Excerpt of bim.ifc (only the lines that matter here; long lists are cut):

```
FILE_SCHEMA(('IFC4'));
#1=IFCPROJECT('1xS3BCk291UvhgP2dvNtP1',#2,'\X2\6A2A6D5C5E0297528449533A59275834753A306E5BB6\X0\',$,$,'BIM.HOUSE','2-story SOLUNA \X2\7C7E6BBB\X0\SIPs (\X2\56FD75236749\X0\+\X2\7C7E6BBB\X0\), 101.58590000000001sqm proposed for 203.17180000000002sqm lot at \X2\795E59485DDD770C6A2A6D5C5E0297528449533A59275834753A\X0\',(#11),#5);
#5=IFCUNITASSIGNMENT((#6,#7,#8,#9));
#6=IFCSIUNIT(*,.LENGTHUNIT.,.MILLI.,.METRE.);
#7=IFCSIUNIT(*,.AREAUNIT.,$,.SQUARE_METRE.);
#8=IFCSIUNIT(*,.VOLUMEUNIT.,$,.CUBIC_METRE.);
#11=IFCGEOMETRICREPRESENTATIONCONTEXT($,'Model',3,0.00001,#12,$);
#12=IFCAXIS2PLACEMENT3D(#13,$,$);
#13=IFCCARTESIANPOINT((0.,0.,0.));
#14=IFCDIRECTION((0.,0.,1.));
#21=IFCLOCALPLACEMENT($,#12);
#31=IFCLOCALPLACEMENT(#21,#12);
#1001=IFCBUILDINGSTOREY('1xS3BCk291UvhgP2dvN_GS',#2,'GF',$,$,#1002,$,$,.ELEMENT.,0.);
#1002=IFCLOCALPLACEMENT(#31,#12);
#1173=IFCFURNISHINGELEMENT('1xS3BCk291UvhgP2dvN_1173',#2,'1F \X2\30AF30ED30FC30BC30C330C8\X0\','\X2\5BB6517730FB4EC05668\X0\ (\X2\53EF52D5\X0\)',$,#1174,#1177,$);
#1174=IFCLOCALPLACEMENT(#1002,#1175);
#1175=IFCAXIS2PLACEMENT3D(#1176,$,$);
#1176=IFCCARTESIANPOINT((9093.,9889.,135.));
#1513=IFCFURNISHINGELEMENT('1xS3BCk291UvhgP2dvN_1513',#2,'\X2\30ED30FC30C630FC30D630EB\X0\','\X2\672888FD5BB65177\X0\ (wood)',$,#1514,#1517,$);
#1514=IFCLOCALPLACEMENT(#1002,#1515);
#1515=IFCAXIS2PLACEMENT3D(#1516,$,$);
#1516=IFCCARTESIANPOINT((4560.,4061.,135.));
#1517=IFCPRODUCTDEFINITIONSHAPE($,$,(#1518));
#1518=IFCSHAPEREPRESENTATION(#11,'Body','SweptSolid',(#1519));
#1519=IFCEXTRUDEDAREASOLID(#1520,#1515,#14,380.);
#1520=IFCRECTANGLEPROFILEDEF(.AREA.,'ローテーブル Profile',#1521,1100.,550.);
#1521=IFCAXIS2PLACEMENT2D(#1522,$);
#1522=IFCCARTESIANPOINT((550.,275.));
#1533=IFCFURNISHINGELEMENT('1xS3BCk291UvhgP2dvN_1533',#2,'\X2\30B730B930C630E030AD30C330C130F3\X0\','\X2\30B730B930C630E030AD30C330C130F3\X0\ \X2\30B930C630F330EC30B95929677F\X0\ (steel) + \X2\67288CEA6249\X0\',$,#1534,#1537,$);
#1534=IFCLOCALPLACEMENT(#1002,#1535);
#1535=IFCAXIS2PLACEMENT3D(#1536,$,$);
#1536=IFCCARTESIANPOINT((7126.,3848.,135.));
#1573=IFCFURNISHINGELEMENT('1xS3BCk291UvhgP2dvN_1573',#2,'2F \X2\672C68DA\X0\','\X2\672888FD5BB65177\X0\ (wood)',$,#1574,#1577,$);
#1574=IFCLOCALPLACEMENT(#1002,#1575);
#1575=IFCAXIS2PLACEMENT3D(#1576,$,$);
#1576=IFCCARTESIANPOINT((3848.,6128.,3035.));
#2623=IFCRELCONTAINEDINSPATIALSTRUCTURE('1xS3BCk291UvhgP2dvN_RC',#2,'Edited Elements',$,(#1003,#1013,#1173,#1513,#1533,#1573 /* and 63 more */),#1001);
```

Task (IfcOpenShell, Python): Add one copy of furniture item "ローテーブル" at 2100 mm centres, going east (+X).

```python
import numpy as np
import ifcopenshell
import ifcopenshell.api.geometry
import ifcopenshell.api.root
import ifcopenshell.util.element
import ifcopenshell.util.placement
import ifcopenshell.util.unit

model = ifcopenshell.open("bim.ifc")
unit_scale = ifcopenshell.util.unit.calculate_unit_scale(model)


def reuse_history(source, copy):
    """copy_class also copies each property set's owner history, people and application; keep the originals."""
    for rel in copy.IsDefinedBy:
        if rel.is_a("IfcRelDefinesByProperties") and (history := rel.RelatingPropertyDefinition.OwnerHistory):
            rel.RelatingPropertyDefinition.OwnerHistory = source.OwnerHistory
            ifcopenshell.util.element.remove_deep2(model, history)


source = model.by_id(1513)
base = ifcopenshell.util.placement.get_local_placement(source.ObjectPlacement)
step = np.array([1.0, 0.0, 0.0]) * 2.1 / unit_scale

for i in range(1, 2):
    copy = ifcopenshell.api.root.copy_class(model, product=source)
    copy.Representation = ifcopenshell.util.element.copy_deep(
        model, source.Representation, exclude=["IfcGeometricRepresentationContext", "IfcRepresentationMap"]
    )
    reuse_history(source, copy)
    matrix = base.copy()
    matrix[:3, 3] += i * step
    print("added at", matrix[:3, 3].round(3) + 0.0)
    ifcopenshell.api.geometry.edit_object_placement(model, product=copy, matrix=matrix, is_si=False)

model.write("bim_edited.ifc")
```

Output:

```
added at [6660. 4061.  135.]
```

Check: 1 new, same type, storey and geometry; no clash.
